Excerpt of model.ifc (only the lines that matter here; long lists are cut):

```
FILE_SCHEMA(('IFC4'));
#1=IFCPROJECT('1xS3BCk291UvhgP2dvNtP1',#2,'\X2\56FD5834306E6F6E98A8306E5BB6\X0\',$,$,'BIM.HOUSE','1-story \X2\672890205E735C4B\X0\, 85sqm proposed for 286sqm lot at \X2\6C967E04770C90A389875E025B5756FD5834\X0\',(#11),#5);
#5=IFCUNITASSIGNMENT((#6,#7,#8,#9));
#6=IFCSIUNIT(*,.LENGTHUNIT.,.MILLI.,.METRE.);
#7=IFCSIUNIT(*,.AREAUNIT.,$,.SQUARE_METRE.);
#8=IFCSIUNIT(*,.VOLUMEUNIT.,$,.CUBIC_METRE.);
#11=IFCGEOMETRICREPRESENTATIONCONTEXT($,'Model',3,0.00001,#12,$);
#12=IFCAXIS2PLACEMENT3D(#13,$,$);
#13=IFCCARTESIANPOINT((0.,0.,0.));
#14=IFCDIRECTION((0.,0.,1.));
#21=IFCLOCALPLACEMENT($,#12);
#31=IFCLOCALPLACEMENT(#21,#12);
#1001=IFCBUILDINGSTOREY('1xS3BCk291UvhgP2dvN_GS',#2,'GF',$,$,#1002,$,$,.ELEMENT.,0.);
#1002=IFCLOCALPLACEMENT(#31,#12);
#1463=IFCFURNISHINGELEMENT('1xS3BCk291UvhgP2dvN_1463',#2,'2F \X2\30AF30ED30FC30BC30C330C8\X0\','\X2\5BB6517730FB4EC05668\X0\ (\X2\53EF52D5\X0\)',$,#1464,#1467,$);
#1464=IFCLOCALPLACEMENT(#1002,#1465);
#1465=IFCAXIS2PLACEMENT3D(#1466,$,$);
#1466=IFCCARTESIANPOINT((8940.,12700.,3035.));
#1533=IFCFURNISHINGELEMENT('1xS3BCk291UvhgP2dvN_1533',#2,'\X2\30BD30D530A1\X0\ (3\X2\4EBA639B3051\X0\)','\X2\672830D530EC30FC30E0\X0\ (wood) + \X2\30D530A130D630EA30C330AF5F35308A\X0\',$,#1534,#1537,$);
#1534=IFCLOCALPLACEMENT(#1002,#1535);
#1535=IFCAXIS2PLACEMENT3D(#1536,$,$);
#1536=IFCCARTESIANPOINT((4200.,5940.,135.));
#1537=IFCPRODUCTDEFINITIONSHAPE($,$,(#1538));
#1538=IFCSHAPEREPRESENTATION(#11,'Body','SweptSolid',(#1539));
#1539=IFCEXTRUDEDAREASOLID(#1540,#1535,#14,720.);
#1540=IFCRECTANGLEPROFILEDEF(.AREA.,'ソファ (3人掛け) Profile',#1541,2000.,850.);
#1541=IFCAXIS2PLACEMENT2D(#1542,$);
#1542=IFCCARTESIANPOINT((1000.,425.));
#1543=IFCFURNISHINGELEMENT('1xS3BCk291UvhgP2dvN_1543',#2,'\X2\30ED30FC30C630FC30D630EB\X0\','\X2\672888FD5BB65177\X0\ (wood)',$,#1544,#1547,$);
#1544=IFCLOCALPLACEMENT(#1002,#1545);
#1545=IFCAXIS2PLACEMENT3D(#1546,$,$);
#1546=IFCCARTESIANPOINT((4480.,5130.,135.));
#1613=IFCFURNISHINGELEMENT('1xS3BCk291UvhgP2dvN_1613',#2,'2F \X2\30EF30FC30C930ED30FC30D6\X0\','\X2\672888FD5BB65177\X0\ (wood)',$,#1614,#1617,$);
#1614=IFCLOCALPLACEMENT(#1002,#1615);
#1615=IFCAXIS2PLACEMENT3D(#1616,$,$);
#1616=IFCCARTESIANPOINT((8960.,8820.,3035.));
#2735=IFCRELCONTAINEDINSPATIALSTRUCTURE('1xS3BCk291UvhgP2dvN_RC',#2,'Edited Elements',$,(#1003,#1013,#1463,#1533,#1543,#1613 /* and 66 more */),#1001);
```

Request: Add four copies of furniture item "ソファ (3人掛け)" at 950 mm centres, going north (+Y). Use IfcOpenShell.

```python
import numpy as np
import ifcopenshell
import ifcopenshell.api.geometry
import ifcopenshell.api.root
import ifcopenshell.util.element
import ifcopenshell.util.placement
import ifcopenshell.util.unit

model = ifcopenshell.open("model.ifc")
unit_scale = ifcopenshell.util.unit.calculate_unit_scale(model)


def reuse_history(source, copy):
    """copy_class also copies each property set's owner history, people and application; keep the originals."""
    for rel in copy.IsDefinedBy:
        if rel.is_a("IfcRelDefinesByProperties") and (history := rel.RelatingPropertyDefinition.OwnerHistory):
            rel.RelatingPropertyDefinition.OwnerHistory = source.OwnerHistory
            ifcopenshell.util.element.remove_deep2(model, history)


source = model.by_guid("1xS3BCk291UvhgP2dvN_1533")
base = ifcopenshell.util.placement.get_local_placement(source.ObjectPlacement)
step = np.array([0.0, 1.0, 0.0]) * 0.95 / unit_scale

for i in range(1, 5):
    copy = ifcopenshell.api.root.copy_class(model, product=source)
    copy.Representation = ifcopenshell.util.element.copy_deep(
        model, source.Representation, exclude=["IfcGeometricRepresentationContext", "IfcRepresentationMap"]
    )
    reuse_history(source, copy)
    matrix = base.copy()
    matrix[:3, 3] += i * step
    print("added at", matrix[:3, 3].round(3) + 0.0)
    ifcopenshell.api.geometry.edit_object_placement(model, product=copy, matrix=matrix, is_si=False)

model.write("model_v2.ifc")
```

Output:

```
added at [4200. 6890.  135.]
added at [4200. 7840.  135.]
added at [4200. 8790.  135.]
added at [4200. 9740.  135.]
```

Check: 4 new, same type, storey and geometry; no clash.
